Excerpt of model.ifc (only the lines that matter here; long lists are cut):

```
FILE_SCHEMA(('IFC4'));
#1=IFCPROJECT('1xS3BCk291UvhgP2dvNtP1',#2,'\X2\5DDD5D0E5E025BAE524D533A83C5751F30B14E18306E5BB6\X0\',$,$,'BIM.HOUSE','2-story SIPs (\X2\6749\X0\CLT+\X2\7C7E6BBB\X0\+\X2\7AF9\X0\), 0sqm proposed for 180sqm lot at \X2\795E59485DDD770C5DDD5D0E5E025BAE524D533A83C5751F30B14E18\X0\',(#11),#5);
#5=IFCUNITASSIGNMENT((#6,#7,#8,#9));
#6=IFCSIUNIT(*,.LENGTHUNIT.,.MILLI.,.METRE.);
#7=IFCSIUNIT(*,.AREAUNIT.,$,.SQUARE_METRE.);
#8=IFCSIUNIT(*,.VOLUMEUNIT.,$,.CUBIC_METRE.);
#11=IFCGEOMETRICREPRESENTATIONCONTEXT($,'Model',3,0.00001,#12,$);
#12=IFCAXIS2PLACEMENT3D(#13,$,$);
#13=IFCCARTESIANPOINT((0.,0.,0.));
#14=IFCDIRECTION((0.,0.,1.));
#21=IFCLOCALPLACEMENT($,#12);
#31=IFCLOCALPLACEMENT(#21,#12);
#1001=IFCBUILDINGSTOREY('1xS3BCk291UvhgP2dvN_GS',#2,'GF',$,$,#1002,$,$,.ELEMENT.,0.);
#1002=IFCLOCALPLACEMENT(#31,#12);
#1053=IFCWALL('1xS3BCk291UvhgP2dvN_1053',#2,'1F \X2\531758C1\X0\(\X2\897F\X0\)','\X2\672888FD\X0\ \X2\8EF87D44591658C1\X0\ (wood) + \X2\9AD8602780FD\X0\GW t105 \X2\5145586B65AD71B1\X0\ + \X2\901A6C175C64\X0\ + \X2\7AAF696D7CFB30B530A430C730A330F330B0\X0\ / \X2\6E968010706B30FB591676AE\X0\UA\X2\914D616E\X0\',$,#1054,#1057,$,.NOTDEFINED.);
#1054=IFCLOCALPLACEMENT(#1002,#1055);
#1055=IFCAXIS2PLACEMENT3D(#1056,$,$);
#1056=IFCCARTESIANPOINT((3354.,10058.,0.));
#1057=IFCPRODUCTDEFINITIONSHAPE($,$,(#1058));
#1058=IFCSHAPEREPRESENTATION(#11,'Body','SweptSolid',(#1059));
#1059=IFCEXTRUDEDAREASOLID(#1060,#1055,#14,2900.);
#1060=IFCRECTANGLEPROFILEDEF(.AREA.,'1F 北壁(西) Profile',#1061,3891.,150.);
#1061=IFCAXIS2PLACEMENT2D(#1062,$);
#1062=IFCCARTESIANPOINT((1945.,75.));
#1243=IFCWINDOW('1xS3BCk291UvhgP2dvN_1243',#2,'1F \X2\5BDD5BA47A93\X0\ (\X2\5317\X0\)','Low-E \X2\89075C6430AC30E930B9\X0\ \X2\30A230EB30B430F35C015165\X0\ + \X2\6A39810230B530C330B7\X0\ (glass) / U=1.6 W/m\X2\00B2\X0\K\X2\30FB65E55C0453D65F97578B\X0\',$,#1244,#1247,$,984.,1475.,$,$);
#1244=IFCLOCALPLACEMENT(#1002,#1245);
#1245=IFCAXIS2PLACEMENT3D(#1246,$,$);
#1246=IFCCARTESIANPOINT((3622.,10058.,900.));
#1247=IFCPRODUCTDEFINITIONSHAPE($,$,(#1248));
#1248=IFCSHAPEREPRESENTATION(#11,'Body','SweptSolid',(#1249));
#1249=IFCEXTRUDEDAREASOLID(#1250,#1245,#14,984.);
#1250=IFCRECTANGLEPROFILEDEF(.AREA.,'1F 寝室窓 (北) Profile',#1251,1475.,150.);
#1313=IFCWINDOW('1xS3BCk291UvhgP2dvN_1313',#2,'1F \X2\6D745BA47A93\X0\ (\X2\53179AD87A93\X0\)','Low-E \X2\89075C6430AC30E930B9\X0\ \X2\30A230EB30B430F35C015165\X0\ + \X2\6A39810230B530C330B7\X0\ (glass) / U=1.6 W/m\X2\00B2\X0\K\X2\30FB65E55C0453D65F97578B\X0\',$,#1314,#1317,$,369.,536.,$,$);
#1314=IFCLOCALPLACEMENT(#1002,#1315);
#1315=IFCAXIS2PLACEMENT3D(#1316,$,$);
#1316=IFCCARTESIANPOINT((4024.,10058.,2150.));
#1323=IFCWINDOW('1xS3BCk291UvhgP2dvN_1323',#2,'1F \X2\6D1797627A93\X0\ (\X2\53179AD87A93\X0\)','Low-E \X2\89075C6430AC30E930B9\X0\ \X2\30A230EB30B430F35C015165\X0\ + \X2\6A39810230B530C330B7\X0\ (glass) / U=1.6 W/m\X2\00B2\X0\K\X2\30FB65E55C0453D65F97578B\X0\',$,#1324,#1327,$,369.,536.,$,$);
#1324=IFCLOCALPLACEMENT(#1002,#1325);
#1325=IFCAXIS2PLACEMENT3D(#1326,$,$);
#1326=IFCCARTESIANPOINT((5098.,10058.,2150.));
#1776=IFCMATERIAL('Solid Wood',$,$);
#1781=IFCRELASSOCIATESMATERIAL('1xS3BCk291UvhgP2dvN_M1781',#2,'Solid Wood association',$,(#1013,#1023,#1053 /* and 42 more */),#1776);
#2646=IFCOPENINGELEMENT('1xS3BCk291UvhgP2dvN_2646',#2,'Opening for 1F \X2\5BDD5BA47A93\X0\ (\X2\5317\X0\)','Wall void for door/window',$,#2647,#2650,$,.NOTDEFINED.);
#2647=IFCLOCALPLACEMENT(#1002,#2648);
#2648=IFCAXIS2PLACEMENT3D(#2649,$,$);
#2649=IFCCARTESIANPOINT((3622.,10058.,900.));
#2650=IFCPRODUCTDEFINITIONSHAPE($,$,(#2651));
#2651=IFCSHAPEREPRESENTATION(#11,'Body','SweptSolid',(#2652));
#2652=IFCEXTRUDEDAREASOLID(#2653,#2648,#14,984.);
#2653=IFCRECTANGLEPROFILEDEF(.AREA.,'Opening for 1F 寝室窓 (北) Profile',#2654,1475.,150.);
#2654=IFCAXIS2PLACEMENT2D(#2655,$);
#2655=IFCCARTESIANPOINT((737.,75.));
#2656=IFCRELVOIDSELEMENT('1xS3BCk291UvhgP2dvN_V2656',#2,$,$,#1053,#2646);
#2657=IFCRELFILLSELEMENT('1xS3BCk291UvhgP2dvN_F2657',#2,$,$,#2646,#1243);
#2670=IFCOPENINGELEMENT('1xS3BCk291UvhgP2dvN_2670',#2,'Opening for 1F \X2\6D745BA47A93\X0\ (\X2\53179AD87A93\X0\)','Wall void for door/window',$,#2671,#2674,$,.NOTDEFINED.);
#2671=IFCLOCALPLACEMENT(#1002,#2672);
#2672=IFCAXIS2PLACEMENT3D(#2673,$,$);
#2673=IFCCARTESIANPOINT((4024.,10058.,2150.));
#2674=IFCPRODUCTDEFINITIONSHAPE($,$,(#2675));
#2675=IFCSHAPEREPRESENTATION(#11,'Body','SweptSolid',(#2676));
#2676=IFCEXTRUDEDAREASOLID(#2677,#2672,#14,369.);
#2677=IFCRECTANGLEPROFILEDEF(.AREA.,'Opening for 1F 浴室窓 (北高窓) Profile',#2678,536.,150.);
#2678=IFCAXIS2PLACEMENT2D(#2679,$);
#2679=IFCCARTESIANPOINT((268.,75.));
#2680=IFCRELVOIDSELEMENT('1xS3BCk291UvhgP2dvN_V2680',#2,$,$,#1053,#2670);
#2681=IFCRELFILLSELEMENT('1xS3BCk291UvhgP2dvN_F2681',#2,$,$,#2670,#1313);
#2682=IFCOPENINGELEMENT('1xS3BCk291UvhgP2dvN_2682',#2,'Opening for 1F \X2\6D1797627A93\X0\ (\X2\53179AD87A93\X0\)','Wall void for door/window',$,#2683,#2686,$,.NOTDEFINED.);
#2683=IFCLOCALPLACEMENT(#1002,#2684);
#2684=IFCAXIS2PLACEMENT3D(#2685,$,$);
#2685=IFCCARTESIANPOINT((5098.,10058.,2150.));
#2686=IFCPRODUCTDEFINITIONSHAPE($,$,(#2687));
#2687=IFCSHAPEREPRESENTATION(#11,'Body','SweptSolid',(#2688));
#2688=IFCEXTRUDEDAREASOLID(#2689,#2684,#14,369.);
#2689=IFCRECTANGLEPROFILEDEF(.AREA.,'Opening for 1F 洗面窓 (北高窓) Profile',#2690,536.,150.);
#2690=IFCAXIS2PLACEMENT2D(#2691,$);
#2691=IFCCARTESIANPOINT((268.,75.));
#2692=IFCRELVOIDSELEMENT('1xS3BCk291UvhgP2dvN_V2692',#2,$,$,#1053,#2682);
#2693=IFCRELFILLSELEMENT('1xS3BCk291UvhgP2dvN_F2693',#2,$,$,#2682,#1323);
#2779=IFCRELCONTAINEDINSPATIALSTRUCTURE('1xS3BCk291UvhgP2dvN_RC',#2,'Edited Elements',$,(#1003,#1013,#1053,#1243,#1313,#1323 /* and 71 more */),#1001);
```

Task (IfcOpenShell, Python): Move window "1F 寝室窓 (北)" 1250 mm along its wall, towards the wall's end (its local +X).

```python
import ifcopenshell
import ifcopenshell.api.geometry
import ifcopenshell.util.placement
import ifcopenshell.util.unit

model = ifcopenshell.open("model.ifc")
unit_scale = ifcopenshell.util.unit.calculate_unit_scale(model)

window = model.by_guid("1xS3BCk291UvhgP2dvN_1243")
opening = window.FillsVoids[0].RelatingOpeningElement
wall = opening.VoidsElements[0].RelatingBuildingElement

wall_matrix = ifcopenshell.util.placement.get_local_placement(wall.ObjectPlacement)
shift = wall_matrix[:3, 0] * 1.25 / unit_scale
before = ifcopenshell.util.placement.get_local_placement(window.ObjectPlacement)[:3, 3].copy()

# The window is not placed relative to its opening, so move both.
for product in (opening, window):
    matrix = ifcopenshell.util.placement.get_local_placement(product.ObjectPlacement)
    matrix[:3, 3] += shift
    ifcopenshell.api.geometry.edit_object_placement(model, product=product, matrix=matrix, is_si=False)

after = ifcopenshell.util.placement.get_local_placement(window.ObjectPlacement)[:3, 3]
print("window moved by", (after - before).round(3) + 0.0)

model.write("model_v2.ifc")
```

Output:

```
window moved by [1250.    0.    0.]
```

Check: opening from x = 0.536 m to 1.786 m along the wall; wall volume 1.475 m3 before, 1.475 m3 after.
